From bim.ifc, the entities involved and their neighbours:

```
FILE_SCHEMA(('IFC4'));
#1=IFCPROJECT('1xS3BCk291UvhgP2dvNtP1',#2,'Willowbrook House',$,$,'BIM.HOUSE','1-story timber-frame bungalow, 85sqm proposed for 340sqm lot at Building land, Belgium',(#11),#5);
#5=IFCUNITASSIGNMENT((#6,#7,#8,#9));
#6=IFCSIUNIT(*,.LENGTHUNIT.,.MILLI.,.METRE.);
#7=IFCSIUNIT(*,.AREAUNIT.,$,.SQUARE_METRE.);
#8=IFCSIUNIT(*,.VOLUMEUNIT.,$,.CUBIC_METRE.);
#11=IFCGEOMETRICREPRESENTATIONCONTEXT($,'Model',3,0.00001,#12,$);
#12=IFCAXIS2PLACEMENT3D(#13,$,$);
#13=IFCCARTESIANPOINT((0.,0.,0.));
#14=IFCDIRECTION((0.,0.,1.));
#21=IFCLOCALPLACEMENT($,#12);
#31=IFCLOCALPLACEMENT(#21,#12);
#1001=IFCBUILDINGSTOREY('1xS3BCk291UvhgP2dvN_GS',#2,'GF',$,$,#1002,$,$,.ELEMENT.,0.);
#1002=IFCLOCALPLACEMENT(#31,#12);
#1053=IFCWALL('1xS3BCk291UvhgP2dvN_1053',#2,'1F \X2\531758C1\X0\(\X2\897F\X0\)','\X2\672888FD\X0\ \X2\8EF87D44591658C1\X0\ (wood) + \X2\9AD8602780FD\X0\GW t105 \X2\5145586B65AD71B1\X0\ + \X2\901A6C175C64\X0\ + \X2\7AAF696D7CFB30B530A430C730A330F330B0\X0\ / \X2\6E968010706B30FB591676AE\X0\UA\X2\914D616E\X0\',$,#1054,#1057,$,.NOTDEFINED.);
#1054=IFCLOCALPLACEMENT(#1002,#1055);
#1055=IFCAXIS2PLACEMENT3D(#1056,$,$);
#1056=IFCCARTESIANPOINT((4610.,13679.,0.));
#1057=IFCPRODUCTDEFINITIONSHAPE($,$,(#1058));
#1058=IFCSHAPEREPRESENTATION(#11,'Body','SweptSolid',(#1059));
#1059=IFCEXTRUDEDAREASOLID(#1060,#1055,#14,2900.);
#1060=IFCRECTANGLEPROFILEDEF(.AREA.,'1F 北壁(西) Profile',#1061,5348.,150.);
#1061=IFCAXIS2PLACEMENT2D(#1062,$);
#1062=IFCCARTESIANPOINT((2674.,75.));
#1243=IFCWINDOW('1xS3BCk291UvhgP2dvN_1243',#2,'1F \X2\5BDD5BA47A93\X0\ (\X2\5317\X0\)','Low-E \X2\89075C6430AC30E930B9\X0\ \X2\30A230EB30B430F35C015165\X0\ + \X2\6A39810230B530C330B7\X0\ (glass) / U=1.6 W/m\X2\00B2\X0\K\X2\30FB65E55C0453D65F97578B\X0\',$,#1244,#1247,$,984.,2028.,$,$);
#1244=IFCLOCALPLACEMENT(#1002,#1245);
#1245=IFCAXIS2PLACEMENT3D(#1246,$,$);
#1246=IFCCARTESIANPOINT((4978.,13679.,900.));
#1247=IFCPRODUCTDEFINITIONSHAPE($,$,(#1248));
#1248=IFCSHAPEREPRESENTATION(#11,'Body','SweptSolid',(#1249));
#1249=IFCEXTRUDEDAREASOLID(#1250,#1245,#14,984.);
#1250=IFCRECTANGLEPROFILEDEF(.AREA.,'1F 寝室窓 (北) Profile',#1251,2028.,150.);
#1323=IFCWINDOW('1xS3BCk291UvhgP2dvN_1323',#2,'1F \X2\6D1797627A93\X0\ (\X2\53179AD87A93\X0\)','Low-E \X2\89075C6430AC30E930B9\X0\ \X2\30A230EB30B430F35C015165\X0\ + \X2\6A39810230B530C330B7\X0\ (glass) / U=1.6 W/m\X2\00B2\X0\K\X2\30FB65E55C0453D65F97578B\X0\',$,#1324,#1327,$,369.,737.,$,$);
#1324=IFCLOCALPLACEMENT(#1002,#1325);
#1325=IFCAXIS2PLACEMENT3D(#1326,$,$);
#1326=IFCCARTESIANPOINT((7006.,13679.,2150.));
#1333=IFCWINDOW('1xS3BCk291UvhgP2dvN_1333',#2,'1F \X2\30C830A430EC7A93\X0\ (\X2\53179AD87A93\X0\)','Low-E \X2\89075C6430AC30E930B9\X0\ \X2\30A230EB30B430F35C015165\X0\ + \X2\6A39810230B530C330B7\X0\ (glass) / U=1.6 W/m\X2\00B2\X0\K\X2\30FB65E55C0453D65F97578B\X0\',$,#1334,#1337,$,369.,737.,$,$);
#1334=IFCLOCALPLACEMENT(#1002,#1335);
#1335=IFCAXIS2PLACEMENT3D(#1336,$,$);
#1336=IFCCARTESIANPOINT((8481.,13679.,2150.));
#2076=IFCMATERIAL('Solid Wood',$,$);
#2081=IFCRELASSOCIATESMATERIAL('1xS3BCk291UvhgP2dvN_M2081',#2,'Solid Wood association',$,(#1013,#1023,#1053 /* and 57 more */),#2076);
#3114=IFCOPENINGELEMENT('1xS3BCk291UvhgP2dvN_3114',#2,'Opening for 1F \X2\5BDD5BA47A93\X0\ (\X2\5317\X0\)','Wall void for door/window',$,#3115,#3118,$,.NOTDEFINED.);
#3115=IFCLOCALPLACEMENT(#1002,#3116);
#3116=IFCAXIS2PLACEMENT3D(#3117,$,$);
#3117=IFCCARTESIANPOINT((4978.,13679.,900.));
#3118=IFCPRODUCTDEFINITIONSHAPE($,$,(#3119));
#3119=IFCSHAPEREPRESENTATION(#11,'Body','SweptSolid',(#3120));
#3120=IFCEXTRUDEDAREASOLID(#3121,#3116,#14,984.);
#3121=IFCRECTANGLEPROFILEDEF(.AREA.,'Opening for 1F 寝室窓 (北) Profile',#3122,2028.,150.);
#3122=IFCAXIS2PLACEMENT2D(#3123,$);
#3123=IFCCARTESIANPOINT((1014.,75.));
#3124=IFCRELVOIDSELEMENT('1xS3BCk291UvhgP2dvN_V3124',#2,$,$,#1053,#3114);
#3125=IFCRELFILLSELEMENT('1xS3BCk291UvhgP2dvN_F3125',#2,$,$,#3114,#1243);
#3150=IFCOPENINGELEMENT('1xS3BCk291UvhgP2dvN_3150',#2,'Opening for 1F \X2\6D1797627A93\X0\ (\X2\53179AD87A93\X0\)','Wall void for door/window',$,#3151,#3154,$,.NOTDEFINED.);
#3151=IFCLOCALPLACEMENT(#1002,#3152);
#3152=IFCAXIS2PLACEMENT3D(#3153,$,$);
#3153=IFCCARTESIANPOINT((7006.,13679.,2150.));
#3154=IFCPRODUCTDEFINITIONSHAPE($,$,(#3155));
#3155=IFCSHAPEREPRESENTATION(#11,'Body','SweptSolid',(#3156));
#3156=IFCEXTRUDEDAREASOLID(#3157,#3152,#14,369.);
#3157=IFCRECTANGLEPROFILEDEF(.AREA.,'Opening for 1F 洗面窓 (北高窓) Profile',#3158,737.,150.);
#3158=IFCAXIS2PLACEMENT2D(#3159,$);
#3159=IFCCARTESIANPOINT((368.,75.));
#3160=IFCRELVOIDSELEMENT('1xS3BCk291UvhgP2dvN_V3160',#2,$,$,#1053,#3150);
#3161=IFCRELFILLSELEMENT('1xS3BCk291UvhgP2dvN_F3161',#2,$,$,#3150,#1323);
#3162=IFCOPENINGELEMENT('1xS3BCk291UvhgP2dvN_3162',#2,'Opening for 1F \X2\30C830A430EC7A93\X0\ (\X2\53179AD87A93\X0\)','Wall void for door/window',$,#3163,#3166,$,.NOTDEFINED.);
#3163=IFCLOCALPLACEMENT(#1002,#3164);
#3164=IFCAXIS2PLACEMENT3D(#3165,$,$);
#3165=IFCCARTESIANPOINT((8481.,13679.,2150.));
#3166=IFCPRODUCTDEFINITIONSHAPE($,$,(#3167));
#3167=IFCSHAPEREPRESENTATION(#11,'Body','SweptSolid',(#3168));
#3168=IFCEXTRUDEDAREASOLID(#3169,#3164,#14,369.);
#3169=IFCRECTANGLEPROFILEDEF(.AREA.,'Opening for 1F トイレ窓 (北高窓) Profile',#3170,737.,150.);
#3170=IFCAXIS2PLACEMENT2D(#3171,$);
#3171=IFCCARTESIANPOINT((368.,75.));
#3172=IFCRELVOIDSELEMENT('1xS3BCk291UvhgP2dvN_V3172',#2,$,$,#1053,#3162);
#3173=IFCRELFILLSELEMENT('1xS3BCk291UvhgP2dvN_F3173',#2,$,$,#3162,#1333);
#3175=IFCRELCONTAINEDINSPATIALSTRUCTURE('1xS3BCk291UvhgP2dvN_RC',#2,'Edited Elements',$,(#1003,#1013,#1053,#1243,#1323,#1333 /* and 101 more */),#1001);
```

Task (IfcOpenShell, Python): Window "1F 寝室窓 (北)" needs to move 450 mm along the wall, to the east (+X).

```python
import ifcopenshell
import ifcopenshell.api.geometry
import ifcopenshell.util.placement

model = ifcopenshell.open("bim.ifc")

window = model.by_id(1243)
opening = window.FillsVoids[0].RelatingOpeningElement
wall = opening.VoidsElements[0].RelatingBuildingElement

wall_matrix = ifcopenshell.util.placement.get_local_placement(wall.ObjectPlacement)
shift = wall_matrix[:3, 0] * 450.0
before = ifcopenshell.util.placement.get_local_placement(window.ObjectPlacement)[:3, 3].copy()

# The window is not placed relative to its opening, so move both.
for product in (opening, window):
    matrix = ifcopenshell.util.placement.get_local_placement(product.ObjectPlacement)
    matrix[:3, 3] += shift
    ifcopenshell.api.geometry.edit_object_placement(model, product=product, matrix=matrix, is_si=False)

after = ifcopenshell.util.placement.get_local_placement(window.ObjectPlacement)[:3, 3]
print("window moved by", (after - before).round(3) + 0.0)

model.write("bim_v2.ifc")
```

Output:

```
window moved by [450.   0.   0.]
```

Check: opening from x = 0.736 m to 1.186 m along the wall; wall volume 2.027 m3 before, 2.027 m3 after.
